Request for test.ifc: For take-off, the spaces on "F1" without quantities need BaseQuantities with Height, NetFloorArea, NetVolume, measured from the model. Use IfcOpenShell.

First a look at what the model holds.

```python
import ifcopenshell
import ifcopenshell.util.element
import ifcopenshell.util.unit

model = ifcopenshell.open("test.ifc")
print(model.schema)
for unit_type in ("LENGTHUNIT", "AREAUNIT", "VOLUMEUNIT"):
    print(unit_type, ifcopenshell.util.unit.calculate_unit_scale(model, unit_type))
storey = next(s for s in model.by_type("IfcBuildingStorey") if s.Name == "F1")
spaces = [e for e in ifcopenshell.util.element.get_decomposition(storey) if e.is_a("IfcSpace")]
for e in sorted(spaces, key=lambda e: e.id()):
    print(e.id(), e.is_a(), e.Name, list(ifcopenshell.util.element.get_psets(e, qtos_only=True)), sep=" | ")
```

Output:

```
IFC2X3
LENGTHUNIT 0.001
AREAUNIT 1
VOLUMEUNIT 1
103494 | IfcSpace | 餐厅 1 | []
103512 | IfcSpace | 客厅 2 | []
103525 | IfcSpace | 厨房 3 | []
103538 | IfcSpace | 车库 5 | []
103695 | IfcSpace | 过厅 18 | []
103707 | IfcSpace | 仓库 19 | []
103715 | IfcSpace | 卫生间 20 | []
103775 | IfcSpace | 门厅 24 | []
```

```python
import ifcopenshell
import ifcopenshell.api.pset
import ifcopenshell.geom
import ifcopenshell.util.element
import ifcopenshell.util.shape
import ifcopenshell.util.unit

model = ifcopenshell.open("test.ifc")
unit_scale = ifcopenshell.util.unit.calculate_unit_scale(model)
area_scale = ifcopenshell.util.unit.calculate_unit_scale(model, "AREAUNIT")
volume_scale = ifcopenshell.util.unit.calculate_unit_scale(model, "VOLUMEUNIT")
settings = ifcopenshell.geom.settings()

storey = next(s for s in model.by_type("IfcBuildingStorey") if s.Name == "F1")
spaces = [e for e in ifcopenshell.util.element.get_decomposition(storey) if e.is_a("IfcSpace")]

for e in sorted(spaces, key=lambda e: e.id()):
    if ifcopenshell.util.element.get_psets(e, qtos_only=True, should_inherit=False):
        continue
    # Geometry comes back in metres, in the element's own axes.
    shape = ifcopenshell.geom.create_shape(settings, e)
    values = {
        "Height": ifcopenshell.util.shape.get_z(shape.geometry) / unit_scale,
        "NetFloorArea": ifcopenshell.util.shape.get_footprint_area(shape.geometry) / area_scale,
        "NetVolume": ifcopenshell.util.shape.get_volume(shape.geometry) / volume_scale,
    }
    qto = ifcopenshell.api.pset.add_qto(model, product=e, name="BaseQuantities")
    ifcopenshell.api.pset.edit_qto(model, qto=qto, properties=values)
    print(e.id(), {k: round(v, 3) for k, v in values.items()})

model.write("test_updated.ifc")
```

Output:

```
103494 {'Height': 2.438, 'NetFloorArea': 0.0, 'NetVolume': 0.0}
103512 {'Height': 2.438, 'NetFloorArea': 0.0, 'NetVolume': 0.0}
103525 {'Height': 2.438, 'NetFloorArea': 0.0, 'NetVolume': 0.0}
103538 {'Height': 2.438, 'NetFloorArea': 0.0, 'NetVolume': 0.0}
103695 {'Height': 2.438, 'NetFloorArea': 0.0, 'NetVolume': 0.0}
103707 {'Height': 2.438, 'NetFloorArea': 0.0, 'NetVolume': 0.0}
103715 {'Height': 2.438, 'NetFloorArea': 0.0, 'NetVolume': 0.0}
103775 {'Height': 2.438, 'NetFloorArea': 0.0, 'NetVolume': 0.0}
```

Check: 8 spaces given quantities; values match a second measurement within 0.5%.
